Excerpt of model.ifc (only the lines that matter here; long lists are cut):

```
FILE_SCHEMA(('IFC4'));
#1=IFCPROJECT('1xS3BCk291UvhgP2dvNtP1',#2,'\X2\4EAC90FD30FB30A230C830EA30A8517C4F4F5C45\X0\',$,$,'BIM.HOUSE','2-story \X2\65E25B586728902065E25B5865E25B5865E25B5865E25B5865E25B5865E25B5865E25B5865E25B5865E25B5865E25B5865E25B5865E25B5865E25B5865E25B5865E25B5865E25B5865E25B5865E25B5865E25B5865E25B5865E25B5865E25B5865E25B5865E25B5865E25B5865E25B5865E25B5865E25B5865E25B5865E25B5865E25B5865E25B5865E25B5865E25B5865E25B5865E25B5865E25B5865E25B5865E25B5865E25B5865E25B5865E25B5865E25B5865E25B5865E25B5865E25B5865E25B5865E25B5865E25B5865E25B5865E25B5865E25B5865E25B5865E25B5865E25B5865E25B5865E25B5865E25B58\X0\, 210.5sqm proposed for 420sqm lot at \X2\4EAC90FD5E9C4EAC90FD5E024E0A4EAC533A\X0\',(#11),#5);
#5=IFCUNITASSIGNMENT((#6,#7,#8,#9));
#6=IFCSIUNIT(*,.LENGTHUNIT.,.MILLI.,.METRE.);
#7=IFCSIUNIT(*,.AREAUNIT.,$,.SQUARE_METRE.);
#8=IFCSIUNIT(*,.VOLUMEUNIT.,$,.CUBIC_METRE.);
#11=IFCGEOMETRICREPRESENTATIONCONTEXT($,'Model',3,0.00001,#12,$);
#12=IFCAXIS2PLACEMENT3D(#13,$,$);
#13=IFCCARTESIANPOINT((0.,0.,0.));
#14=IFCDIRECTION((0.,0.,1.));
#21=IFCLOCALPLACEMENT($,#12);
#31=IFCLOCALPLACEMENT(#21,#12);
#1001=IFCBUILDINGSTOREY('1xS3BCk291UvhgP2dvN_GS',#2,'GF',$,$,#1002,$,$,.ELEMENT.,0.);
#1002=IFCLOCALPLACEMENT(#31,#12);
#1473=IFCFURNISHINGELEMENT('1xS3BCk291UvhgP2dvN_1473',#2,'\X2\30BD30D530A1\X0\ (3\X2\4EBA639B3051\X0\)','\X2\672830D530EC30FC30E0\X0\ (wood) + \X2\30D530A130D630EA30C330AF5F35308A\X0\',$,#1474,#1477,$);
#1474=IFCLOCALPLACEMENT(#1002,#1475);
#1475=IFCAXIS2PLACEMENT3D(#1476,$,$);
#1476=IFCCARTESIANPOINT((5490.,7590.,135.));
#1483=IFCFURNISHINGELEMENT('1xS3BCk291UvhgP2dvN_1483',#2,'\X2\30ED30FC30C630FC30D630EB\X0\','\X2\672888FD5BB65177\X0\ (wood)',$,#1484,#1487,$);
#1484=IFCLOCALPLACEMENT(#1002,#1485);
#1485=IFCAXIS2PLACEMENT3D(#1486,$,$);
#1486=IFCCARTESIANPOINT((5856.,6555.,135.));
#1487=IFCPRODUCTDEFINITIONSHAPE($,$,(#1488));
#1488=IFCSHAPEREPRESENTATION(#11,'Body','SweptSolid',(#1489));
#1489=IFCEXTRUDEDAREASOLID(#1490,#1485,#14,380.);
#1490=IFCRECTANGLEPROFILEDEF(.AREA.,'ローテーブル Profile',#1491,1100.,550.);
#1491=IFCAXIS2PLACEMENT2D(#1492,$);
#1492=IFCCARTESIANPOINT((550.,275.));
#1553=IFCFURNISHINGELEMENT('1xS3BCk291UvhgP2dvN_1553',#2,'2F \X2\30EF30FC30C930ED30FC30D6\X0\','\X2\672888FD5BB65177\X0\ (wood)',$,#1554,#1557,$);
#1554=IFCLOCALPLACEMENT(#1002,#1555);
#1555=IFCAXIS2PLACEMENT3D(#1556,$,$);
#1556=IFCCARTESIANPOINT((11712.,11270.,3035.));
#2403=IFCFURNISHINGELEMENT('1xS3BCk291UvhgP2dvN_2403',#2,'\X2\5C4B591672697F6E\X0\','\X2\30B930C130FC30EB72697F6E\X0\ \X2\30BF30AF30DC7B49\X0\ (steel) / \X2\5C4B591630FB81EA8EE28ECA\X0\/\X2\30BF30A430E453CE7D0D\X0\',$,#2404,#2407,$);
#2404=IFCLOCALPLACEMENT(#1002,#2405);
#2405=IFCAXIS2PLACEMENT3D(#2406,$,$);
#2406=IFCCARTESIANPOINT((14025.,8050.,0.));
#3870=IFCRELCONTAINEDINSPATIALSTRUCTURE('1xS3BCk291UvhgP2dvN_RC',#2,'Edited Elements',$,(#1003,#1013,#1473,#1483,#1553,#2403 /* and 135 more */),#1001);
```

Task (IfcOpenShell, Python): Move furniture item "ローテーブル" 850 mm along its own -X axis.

```python
import ifcopenshell
import ifcopenshell.api.geometry
import ifcopenshell.util.placement
import ifcopenshell.util.unit

model = ifcopenshell.open("model.ifc")
unit_scale = ifcopenshell.util.unit.calculate_unit_scale(model)

item = model.by_guid("1xS3BCk291UvhgP2dvN_1483")
matrix = ifcopenshell.util.placement.get_local_placement(item.ObjectPlacement)
matrix[:3, 3] -= matrix[:3, 0] * 0.85 / unit_scale
ifcopenshell.api.geometry.edit_object_placement(model, product=item, matrix=matrix, is_si=False)

print(ifcopenshell.util.placement.get_local_placement(item.ObjectPlacement).round(3) + 0.0)

model.write("model_edited.ifc")
```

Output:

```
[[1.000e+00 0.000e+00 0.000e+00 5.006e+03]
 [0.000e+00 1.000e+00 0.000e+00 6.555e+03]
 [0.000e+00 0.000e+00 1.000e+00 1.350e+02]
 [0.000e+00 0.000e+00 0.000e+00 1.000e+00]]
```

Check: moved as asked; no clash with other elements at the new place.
